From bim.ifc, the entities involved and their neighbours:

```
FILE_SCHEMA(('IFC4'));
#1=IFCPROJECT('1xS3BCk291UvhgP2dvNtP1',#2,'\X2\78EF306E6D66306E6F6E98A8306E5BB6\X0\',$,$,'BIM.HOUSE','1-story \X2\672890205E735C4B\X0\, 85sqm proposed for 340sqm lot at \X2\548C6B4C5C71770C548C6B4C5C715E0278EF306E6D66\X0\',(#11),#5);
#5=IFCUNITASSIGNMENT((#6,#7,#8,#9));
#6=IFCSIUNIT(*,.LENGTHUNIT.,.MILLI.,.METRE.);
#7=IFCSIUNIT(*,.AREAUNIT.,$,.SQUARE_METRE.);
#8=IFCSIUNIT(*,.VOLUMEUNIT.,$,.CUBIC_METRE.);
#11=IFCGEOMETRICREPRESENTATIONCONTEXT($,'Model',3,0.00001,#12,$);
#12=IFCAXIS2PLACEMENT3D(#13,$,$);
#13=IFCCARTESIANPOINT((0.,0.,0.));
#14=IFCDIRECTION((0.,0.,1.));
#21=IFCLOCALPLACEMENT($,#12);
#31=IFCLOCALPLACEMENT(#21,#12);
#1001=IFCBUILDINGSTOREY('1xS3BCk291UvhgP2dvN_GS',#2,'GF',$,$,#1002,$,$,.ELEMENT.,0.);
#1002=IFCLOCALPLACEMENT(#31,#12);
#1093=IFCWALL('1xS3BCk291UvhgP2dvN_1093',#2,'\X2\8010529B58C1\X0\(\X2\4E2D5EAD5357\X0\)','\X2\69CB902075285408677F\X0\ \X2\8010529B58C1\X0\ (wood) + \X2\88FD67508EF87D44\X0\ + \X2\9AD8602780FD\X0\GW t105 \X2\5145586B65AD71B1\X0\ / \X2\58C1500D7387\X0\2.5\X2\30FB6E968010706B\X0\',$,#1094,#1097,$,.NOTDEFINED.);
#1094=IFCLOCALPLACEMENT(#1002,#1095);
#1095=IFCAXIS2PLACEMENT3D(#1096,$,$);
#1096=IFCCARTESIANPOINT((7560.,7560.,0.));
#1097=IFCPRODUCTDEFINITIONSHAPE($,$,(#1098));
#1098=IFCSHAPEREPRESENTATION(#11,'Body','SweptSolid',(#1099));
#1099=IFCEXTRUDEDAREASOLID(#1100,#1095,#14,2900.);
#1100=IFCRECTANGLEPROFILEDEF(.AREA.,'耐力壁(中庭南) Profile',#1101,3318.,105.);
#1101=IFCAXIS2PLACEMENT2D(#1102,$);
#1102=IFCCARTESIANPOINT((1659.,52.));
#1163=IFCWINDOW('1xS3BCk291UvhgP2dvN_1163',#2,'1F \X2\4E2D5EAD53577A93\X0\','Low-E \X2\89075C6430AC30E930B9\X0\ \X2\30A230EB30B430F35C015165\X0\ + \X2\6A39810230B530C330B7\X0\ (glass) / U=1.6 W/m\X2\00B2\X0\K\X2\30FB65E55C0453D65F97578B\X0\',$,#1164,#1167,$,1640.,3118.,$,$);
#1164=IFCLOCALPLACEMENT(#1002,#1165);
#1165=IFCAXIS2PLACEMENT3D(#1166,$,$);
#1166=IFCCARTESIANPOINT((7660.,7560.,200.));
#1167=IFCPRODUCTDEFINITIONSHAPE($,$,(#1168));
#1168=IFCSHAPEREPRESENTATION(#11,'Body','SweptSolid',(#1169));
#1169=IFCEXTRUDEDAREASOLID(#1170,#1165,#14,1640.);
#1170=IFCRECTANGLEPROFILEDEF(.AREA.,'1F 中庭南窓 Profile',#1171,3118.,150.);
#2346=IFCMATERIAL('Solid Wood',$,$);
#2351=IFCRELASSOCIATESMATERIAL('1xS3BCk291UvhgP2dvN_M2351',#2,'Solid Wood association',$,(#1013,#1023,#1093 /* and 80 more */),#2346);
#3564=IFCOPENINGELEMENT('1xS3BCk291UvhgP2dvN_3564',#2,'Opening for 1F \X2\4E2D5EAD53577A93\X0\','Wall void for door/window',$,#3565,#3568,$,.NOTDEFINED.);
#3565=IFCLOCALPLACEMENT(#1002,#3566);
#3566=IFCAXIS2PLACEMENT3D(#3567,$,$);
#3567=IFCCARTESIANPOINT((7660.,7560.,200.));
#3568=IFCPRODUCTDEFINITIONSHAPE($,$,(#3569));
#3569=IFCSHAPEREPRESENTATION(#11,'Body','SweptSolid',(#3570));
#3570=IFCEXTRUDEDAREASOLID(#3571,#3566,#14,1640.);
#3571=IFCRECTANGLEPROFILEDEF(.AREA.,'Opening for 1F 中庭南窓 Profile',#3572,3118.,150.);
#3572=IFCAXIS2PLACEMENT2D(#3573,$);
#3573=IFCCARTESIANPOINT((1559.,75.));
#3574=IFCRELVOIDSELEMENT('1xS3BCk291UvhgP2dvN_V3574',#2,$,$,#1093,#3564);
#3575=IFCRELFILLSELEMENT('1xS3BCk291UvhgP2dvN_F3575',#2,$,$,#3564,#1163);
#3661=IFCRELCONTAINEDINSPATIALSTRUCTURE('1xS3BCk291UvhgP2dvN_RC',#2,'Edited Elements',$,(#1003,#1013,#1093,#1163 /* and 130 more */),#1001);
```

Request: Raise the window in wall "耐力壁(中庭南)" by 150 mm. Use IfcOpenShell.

```python
import numpy as np
import ifcopenshell
import ifcopenshell.api.geometry
import ifcopenshell.util.placement
import ifcopenshell.util.unit

model = ifcopenshell.open("bim.ifc")
unit_scale = ifcopenshell.util.unit.calculate_unit_scale(model)

window = model.by_id(1163)
opening = window.FillsVoids[0].RelatingOpeningElement
dz = 0.15 / unit_scale

shift = np.array([0.0, 0.0, dz])
# The window is not placed relative to its opening, so move both.
for product in (opening, window):
    matrix = ifcopenshell.util.placement.get_local_placement(product.ObjectPlacement)
    matrix[:3, 3] += shift
    ifcopenshell.api.geometry.edit_object_placement(model, product=product, matrix=matrix, is_si=False)

print(f"moved by {dz * unit_scale:+.3f} m")

model.write("bim_updated.ifc")
```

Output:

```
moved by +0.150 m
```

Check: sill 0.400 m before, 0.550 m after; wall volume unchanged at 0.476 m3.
